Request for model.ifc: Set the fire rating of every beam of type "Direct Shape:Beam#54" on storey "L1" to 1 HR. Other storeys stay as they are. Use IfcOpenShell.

First a look at what the model holds.

```python
import ifcopenshell
import ifcopenshell.util.element

model = ifcopenshell.open("model.ifc")
print(model.schema)
storey = next(s for s in model.by_type("IfcBuildingStorey") if s.Name == "L1")
beams = [e for e in ifcopenshell.util.element.get_decomposition(storey) if e.is_a("IfcBeam")]
seen = {}
for e in beams:
    element_type = ifcopenshell.util.element.get_type(e)
    key = (element_type.Name if element_type != e and element_type else None, ifcopenshell.util.element.get_pset(e, "Pset_BeamCommon", "FireRating"))
    seen[key] = seen.get(key, 0) + 1
for (name, value), count in sorted(seen.items(), key=str):
    print(count, "x", name, "|", value)
```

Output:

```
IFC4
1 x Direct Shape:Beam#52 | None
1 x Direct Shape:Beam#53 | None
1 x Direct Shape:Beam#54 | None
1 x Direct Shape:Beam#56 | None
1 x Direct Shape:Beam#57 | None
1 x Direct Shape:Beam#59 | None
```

```python
import ifcopenshell
import ifcopenshell.api.pset
import ifcopenshell.util.element

model = ifcopenshell.open("model.ifc")

storey = next(s for s in model.by_type("IfcBuildingStorey") if s.Name == "L1")
beams = [e for e in ifcopenshell.util.element.get_decomposition(storey) if e.is_a("IfcBeam")]

count = 0
for e in beams:
    element_type = ifcopenshell.util.element.get_type(e)
    if element_type in (None, e) or element_type.Name != "Direct Shape:Beam#54":
        continue
    # add_pset returns the element's existing set when there is one.
    pset = ifcopenshell.api.pset.add_pset(model, product=e, name="Pset_BeamCommon")
    ifcopenshell.api.pset.edit_pset(model, pset=pset, properties={"FireRating": "1 HR"})
    count += 1

print(count, "beams updated")

model.write("model_edited.ifc")
```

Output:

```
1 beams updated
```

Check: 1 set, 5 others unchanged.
